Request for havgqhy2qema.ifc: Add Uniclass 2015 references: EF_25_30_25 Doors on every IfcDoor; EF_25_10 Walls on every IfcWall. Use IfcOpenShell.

First a look at what the model holds.

```python
import ifcopenshell

model = ifcopenshell.open("havgqhy2qema.ifc")
print(model.schema)
print("classifications:", [c.Name for c in model.by_type("IfcClassification")])
for ifc_class in ("IfcDoor", "IfcRoof", "IfcStair", "IfcWall", "IfcWindow"):
    print(ifc_class, len(model.by_type(ifc_class)))
```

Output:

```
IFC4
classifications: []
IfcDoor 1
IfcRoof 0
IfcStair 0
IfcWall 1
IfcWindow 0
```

```python
import ifcopenshell
import ifcopenshell.api.classification

model = ifcopenshell.open("havgqhy2qema.ifc")

system = ifcopenshell.api.classification.add_classification(model, classification="Uniclass 2015")

codes = {
    "IfcDoor": ("EF_25_30_25", "Doors"),
    "IfcWall": ("EF_25_10", "Walls"),
}
for ifc_class, (code, name) in codes.items():
    products = model.by_type(ifc_class)
    ifcopenshell.api.classification.add_reference(
        model, products=products, classification=system, identification=code, name=name
    )
    print(code, len(products))

model.write("havgqhy2qema_rev.ifc")
```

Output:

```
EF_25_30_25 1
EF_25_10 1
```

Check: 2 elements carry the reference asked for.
